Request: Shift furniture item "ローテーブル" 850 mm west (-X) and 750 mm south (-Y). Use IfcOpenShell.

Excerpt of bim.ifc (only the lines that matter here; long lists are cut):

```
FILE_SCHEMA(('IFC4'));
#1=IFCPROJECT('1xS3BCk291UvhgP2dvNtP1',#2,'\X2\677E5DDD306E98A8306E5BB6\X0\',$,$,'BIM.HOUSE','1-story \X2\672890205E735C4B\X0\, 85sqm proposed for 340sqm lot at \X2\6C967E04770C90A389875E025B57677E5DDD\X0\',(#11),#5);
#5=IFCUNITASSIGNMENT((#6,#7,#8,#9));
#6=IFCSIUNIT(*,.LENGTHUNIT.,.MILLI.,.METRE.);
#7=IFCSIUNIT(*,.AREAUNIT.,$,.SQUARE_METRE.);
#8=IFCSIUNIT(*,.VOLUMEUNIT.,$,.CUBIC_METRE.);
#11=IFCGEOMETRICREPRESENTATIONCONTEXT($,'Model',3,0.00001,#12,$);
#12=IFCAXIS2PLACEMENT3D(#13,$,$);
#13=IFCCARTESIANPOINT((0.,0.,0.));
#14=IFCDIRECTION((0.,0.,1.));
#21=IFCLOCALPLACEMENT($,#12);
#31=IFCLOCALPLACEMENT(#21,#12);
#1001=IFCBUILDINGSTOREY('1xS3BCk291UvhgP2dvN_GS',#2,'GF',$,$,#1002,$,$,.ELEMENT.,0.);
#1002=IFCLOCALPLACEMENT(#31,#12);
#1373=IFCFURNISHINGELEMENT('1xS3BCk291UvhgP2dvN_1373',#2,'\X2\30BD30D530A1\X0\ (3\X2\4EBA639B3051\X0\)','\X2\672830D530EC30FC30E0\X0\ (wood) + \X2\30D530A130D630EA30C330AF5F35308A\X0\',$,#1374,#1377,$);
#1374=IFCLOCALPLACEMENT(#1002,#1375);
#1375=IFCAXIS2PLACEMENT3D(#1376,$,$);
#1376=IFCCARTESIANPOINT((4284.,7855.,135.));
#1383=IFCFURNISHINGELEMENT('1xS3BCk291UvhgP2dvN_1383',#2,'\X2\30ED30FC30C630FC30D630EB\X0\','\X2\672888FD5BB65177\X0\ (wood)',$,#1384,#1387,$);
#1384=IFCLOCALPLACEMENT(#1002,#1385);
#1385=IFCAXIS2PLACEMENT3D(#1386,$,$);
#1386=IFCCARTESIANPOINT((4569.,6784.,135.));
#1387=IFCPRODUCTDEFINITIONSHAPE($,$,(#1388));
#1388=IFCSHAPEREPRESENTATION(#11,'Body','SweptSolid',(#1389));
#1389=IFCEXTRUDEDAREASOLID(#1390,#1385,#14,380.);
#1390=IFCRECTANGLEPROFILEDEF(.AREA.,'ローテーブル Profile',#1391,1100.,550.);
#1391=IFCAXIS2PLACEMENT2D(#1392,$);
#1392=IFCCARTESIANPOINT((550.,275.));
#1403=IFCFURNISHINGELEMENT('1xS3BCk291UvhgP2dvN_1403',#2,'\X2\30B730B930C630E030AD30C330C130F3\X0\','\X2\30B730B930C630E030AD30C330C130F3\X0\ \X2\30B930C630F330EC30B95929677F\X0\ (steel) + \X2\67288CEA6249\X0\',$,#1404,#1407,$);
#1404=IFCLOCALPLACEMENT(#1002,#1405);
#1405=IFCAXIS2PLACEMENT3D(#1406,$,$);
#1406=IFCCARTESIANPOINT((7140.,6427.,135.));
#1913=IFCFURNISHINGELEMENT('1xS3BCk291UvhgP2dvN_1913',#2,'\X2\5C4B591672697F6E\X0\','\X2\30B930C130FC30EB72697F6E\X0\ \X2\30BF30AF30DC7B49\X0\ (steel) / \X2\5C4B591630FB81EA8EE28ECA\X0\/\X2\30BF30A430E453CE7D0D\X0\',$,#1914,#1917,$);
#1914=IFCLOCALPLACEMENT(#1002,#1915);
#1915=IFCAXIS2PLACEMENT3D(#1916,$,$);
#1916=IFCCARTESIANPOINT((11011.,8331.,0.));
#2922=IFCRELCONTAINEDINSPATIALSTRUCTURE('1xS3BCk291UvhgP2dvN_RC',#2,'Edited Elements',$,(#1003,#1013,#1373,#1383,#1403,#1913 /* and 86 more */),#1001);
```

```python
import ifcopenshell
import ifcopenshell.api.geometry
import ifcopenshell.util.placement
import ifcopenshell.util.unit

model = ifcopenshell.open("bim.ifc")
unit_scale = ifcopenshell.util.unit.calculate_unit_scale(model)

item = model.by_guid("1xS3BCk291UvhgP2dvN_1383")
matrix = ifcopenshell.util.placement.get_local_placement(item.ObjectPlacement)
matrix[0, 3] -= 0.85 / unit_scale
matrix[1, 3] -= 0.75 / unit_scale
ifcopenshell.api.geometry.edit_object_placement(model, product=item, matrix=matrix, is_si=False)

print(ifcopenshell.util.placement.get_local_placement(item.ObjectPlacement).round(3) + 0.0)

model.write("bim_rev.ifc")
```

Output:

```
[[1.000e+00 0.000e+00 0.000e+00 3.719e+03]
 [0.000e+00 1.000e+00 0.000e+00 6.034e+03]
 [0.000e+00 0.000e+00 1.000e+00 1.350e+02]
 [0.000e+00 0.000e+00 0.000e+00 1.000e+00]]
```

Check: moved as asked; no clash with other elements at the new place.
